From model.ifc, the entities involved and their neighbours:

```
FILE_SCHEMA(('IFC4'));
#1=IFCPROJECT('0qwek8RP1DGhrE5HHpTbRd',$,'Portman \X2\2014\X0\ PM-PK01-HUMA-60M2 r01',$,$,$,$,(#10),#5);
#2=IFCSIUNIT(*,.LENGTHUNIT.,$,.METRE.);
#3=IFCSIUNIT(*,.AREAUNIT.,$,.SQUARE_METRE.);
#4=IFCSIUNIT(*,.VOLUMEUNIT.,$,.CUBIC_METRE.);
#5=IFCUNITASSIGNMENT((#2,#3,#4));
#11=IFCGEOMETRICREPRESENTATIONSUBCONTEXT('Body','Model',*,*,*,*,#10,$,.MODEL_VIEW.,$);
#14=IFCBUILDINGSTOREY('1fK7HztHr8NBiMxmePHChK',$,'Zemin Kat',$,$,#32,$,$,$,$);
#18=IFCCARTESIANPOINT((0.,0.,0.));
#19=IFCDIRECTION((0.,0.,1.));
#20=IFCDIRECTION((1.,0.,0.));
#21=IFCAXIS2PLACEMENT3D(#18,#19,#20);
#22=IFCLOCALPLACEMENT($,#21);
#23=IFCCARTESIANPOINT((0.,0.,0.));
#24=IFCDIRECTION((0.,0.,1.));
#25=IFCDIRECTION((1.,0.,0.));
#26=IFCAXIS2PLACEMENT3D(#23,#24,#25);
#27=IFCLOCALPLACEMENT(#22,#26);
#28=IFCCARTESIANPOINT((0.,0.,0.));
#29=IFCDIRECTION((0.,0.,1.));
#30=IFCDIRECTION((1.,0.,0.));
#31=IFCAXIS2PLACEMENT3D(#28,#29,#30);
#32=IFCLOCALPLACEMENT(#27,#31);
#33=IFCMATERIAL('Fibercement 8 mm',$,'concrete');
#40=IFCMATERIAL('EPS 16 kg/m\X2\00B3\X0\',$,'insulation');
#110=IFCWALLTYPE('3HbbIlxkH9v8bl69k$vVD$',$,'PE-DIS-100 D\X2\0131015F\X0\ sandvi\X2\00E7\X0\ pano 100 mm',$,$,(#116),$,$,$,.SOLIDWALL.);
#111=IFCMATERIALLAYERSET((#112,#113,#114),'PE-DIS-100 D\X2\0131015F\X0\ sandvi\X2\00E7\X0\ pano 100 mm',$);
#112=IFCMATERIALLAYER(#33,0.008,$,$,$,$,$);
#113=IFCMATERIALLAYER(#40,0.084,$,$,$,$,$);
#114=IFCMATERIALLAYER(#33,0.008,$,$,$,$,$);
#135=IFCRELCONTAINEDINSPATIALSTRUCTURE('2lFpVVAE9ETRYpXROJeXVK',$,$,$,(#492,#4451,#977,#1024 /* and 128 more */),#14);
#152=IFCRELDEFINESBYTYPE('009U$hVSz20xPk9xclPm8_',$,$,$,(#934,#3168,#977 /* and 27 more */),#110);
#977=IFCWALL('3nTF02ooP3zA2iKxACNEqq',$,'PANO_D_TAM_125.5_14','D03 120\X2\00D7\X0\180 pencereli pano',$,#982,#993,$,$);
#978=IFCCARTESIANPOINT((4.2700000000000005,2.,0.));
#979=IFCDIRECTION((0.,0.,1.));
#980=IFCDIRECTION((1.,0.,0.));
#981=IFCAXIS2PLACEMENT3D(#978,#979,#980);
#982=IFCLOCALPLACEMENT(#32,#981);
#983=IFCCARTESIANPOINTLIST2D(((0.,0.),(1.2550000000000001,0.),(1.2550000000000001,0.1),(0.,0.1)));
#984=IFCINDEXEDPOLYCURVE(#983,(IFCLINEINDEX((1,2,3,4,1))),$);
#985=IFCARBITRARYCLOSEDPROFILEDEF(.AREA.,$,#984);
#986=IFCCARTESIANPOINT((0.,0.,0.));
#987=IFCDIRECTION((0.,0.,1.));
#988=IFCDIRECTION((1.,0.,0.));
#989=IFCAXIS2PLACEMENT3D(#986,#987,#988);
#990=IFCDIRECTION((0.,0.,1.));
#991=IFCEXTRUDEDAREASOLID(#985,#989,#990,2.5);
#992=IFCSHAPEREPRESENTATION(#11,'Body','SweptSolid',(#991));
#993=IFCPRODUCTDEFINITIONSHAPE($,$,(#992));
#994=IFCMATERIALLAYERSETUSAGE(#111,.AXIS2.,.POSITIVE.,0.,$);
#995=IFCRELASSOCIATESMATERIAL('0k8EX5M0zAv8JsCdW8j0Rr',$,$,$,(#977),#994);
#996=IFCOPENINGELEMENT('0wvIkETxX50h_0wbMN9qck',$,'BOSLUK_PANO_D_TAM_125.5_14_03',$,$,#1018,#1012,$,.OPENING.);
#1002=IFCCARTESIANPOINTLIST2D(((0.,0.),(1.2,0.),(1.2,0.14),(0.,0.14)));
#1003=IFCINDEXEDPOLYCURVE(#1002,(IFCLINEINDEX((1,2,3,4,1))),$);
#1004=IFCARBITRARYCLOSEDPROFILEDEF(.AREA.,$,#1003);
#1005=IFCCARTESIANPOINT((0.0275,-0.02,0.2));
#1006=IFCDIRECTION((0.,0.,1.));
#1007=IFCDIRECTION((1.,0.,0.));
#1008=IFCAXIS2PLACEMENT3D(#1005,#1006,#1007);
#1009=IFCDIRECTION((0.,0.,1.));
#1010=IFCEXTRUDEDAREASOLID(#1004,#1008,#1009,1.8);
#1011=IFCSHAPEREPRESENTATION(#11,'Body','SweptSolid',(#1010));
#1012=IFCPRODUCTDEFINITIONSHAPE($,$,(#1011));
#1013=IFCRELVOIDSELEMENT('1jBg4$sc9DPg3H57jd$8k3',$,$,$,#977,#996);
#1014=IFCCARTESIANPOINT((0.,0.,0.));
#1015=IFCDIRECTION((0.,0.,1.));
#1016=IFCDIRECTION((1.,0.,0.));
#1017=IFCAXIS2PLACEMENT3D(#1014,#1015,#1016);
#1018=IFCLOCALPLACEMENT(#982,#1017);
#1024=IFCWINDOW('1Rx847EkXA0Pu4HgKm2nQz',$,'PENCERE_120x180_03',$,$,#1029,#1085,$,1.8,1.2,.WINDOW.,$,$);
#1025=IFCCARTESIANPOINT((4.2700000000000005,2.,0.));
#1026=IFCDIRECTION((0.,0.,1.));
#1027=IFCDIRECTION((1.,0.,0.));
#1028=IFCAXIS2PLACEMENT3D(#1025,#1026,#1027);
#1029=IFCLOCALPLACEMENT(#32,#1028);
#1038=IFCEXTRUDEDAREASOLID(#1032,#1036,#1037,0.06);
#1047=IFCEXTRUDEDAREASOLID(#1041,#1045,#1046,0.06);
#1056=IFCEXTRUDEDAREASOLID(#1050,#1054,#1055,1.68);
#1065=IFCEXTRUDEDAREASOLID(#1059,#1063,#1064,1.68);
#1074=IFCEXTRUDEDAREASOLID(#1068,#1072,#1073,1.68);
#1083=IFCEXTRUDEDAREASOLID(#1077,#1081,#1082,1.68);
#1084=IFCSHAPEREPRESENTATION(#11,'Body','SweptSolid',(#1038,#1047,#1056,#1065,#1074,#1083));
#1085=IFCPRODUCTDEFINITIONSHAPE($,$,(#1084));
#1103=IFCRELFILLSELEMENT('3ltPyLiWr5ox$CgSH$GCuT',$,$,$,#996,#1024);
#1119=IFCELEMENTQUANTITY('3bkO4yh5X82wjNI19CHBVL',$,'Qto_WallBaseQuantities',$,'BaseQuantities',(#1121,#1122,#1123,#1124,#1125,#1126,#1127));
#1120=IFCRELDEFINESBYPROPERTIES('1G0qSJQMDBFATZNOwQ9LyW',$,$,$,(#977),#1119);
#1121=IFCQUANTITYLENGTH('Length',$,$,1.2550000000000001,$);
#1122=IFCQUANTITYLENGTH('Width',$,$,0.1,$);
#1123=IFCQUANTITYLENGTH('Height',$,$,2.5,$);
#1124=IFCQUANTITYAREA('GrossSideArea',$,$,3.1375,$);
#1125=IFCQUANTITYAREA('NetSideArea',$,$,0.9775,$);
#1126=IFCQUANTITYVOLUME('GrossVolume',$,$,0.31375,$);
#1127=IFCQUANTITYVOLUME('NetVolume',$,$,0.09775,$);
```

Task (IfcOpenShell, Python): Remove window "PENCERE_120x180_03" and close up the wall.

```python
import ifcopenshell
import ifcopenshell.api.feature
import ifcopenshell.api.pset
import ifcopenshell.api.root
import ifcopenshell.geom
import ifcopenshell.util.element
import ifcopenshell.util.shape
import ifcopenshell.util.unit

model = ifcopenshell.open("model.ifc")
area_scale = ifcopenshell.util.unit.calculate_unit_scale(model, "AREAUNIT")
volume_scale = ifcopenshell.util.unit.calculate_unit_scale(model, "VOLUMEUNIT")
settings = ifcopenshell.geom.settings()


def volume(element):
    """Net volume in cubic metres, openings subtracted."""
    shape = ifcopenshell.geom.create_shape(settings, element)
    return ifcopenshell.util.shape.get_volume(shape.geometry)


window = model.by_id(1024)
opening = window.FillsVoids[0].RelatingOpeningElement
wall = opening.VoidsElements[0].RelatingBuildingElement
before = volume(wall)

ifcopenshell.api.root.remove_product(model, product=window)
ifcopenshell.api.feature.remove_feature(model, feature=opening)

after = volume(wall)
thickness = 0.1  # wall thickness in metres

# Update the wall's stored quantities.
qto = model.by_id(ifcopenshell.util.element.get_pset(wall, "Qto_WallBaseQuantities", should_inherit=False)["id"])
ifcopenshell.api.pset.edit_qto(model, qto=qto, properties={
    "NetSideArea": after / thickness / area_scale,
    "NetVolume": after / volume_scale,
})

print(f"wall volume {before:.3f} -> {after:.3f} m3")

model.write("model_v2.ifc")
```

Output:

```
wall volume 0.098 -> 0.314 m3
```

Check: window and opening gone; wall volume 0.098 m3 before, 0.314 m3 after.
